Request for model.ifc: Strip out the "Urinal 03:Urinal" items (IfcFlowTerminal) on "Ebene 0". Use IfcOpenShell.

First a look at what the model holds.

```python
import ifcopenshell
import ifcopenshell.util.element

model = ifcopenshell.open("model.ifc")
print(model.schema)
storey = next(s for s in model.by_type("IfcBuildingStorey") if s.Name == "Ebene 0")
terminals = [e for e in ifcopenshell.util.element.get_decomposition(storey) if e.is_a("IfcFlowTerminal")]
seen = {}
for e in terminals:
    element_type = ifcopenshell.util.element.get_type(e)
    name = element_type.Name if element_type not in (None, e) else None
    seen[name] = seen.get(name, 0) + 1
for name, count in sorted(seen.items(), key=str):
    print(count, "x", name)
```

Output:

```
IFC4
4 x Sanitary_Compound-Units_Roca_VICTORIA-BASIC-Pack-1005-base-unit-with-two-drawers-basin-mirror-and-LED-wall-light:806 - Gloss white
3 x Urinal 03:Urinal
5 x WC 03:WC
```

```python
import ifcopenshell
import ifcopenshell.api.root
import ifcopenshell.util.element

model = ifcopenshell.open("model.ifc")

storey = next(s for s in model.by_type("IfcBuildingStorey") if s.Name == "Ebene 0")
terminals = [e for e in ifcopenshell.util.element.get_decomposition(storey) if e.is_a("IfcFlowTerminal")]
targets = [e for e in terminals if (t := ifcopenshell.util.element.get_type(e)) not in (None, e) and t.Name == "Urinal 03:Urinal"]

for e in targets:
    ifcopenshell.api.root.remove_product(model, product=e)
print(len(targets), "removed")

model.write("model_v2.ifc")
```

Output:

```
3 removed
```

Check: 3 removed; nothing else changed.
